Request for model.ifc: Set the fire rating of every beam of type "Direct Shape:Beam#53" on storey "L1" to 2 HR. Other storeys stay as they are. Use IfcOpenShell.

First a look at what the model holds.

```python
import ifcopenshell
import ifcopenshell.util.element

model = ifcopenshell.open("model.ifc")
print(model.schema)
storey = next(s for s in model.by_type("IfcBuildingStorey") if s.Name == "L1")
beams = [e for e in ifcopenshell.util.element.get_decomposition(storey) if e.is_a("IfcBeam")]
seen = {}
for e in beams:
    element_type = ifcopenshell.util.element.get_type(e)
    key = (element_type.Name if element_type != e and element_type else None, ifcopenshell.util.element.get_pset(e, "Pset_BeamCommon", "FireRating"))
    seen[key] = seen.get(key, 0) + 1
for (name, value), count in sorted(seen.items(), key=str):
    print(count, "x", name, "|", value)
```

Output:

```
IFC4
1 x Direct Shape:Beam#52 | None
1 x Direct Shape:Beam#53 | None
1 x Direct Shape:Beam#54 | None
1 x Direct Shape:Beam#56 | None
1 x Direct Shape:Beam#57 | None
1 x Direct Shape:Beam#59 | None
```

```python
import ifcopenshell
import ifcopenshell.api.pset
import ifcopenshell.util.element

model = ifcopenshell.open("model.ifc")

storey = next(s for s in model.by_type("IfcBuildingStorey") if s.Name == "L1")
beams = [e for e in ifcopenshell.util.element.get_decomposition(storey) if e.is_a("IfcBeam")]

count = 0
for e in beams:
    element_type = ifcopenshell.util.element.get_type(e)
    if element_type in (None, e) or element_type.Name != "Direct Shape:Beam#53":
        continue
    # add_pset returns the element's existing set when there is one.
    pset = ifcopenshell.api.pset.add_pset(model, product=e, name="Pset_BeamCommon")
    ifcopenshell.api.pset.edit_pset(model, pset=pset, properties={"FireRating": "2 HR"})
    count += 1

print(count, "beams updated")

model.write("model_updated.ifc")
```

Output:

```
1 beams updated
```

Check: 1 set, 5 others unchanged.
